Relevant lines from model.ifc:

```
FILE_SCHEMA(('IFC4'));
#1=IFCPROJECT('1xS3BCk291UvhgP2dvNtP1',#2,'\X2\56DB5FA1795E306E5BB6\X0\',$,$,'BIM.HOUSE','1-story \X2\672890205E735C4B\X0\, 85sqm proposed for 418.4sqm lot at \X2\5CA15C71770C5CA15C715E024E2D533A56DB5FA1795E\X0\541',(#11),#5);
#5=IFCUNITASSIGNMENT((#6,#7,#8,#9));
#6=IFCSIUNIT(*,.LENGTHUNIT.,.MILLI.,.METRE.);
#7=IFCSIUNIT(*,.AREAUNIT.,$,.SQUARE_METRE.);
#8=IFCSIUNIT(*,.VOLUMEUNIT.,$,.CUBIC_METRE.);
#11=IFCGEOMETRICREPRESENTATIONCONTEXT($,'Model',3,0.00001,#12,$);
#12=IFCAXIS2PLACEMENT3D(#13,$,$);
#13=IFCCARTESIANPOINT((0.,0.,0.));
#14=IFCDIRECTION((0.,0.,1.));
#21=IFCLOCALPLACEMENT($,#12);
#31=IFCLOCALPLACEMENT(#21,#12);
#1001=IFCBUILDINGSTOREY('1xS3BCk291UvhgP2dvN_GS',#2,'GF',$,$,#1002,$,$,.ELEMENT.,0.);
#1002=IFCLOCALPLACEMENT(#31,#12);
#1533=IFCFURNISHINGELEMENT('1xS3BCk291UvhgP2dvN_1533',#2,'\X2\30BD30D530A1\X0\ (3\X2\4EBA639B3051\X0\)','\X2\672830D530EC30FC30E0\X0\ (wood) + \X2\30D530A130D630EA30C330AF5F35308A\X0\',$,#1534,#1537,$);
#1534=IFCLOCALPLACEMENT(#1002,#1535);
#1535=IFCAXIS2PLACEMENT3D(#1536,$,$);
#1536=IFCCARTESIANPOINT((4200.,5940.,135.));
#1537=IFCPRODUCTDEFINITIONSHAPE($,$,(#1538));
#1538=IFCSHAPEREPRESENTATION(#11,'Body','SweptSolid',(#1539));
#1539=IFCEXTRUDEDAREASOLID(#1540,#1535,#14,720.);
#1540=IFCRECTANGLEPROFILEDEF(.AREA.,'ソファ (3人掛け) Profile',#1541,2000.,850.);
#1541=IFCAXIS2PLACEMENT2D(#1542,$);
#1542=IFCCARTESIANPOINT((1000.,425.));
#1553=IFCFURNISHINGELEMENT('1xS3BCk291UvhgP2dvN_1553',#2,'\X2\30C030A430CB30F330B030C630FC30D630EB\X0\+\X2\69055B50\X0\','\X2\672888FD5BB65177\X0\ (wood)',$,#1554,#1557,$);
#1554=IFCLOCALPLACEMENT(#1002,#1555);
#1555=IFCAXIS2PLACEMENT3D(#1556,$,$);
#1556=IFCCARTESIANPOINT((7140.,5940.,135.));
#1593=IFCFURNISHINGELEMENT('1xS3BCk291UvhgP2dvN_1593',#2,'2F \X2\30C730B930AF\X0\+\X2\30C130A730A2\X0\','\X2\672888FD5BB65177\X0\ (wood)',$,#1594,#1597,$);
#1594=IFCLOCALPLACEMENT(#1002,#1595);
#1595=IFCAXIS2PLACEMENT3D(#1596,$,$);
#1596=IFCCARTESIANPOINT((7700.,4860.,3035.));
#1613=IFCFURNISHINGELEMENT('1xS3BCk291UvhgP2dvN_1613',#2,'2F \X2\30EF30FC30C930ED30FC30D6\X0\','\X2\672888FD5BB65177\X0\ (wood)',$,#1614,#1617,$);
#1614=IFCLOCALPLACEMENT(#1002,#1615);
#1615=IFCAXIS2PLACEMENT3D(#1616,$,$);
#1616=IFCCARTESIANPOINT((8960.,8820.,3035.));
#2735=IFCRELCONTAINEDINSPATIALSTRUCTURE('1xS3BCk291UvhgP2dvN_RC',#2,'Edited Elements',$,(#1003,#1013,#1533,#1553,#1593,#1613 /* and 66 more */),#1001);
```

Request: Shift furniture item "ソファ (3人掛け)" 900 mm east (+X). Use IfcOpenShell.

```python
import ifcopenshell
import ifcopenshell.api.geometry
import ifcopenshell.util.placement
import ifcopenshell.util.unit

model = ifcopenshell.open("model.ifc")
unit_scale = ifcopenshell.util.unit.calculate_unit_scale(model)

item = model.by_guid("1xS3BCk291UvhgP2dvN_1533")
matrix = ifcopenshell.util.placement.get_local_placement(item.ObjectPlacement)
matrix[0, 3] += 0.9 / unit_scale
ifcopenshell.api.geometry.edit_object_placement(model, product=item, matrix=matrix, is_si=False)

print(ifcopenshell.util.placement.get_local_placement(item.ObjectPlacement).round(3) + 0.0)

model.write("model_updated.ifc")
```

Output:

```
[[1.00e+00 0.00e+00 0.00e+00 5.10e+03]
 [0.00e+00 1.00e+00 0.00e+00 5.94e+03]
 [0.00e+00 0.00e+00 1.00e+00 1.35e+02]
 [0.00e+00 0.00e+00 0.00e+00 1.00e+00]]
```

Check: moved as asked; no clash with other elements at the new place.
